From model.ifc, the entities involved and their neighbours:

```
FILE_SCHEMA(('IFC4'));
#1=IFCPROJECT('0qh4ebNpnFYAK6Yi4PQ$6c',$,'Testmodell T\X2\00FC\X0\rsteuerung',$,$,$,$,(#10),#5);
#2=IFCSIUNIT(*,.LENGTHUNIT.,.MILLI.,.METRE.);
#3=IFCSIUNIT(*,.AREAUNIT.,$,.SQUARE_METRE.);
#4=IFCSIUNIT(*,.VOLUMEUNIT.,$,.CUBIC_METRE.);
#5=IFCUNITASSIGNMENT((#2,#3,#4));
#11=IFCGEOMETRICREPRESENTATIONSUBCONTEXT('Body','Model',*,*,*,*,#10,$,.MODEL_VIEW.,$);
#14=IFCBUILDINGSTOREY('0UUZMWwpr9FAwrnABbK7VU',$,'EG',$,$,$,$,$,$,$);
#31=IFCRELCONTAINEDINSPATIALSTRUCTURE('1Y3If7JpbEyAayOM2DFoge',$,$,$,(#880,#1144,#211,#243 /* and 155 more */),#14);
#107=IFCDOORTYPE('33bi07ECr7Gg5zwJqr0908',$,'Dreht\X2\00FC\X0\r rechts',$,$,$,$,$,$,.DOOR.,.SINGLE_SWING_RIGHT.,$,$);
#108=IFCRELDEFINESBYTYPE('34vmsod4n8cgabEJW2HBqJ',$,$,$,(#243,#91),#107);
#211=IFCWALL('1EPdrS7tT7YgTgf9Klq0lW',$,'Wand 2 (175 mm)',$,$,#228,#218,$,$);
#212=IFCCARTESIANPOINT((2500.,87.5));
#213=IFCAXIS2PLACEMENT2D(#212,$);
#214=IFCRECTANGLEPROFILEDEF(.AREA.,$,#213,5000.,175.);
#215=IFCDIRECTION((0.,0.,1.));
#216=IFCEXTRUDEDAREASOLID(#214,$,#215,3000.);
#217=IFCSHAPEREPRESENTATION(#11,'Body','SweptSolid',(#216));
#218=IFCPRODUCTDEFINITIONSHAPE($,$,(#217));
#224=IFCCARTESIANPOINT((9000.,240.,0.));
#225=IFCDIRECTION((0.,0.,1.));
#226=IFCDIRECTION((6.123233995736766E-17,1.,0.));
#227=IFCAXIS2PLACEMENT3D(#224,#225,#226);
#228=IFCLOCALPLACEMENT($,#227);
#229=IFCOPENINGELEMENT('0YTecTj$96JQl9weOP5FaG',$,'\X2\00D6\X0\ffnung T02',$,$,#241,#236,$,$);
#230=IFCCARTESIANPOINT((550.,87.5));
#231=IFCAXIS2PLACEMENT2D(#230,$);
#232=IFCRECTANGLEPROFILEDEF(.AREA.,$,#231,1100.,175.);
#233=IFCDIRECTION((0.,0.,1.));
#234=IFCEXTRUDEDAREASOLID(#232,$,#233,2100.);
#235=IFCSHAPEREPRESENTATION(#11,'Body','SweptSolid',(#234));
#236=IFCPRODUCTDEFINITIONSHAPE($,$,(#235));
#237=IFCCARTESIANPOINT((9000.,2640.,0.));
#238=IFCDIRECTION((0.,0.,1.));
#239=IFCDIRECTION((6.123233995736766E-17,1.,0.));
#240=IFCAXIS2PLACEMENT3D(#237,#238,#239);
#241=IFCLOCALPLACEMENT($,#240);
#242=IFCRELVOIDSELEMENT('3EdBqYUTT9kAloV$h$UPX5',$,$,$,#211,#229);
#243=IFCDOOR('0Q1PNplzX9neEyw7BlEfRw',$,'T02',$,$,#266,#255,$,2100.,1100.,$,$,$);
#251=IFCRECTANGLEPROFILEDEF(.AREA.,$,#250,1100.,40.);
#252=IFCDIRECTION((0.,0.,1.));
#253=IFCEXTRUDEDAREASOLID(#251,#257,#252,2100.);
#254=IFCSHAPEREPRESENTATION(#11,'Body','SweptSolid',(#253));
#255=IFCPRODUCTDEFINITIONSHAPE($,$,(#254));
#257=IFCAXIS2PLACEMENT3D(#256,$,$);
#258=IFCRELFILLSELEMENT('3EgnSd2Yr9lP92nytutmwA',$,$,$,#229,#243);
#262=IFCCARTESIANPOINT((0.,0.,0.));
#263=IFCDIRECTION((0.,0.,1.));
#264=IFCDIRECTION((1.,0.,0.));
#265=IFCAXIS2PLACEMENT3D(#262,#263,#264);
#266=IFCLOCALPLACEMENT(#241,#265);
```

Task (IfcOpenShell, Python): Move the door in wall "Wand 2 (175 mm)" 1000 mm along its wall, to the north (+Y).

```python
import ifcopenshell
import ifcopenshell.api.geometry
import ifcopenshell.util.placement
import ifcopenshell.util.unit

model = ifcopenshell.open("model.ifc")
unit_scale = ifcopenshell.util.unit.calculate_unit_scale(model)

door = model.by_guid("0Q1PNplzX9neEyw7BlEfRw")
opening = door.FillsVoids[0].RelatingOpeningElement
wall = opening.VoidsElements[0].RelatingBuildingElement

wall_matrix = ifcopenshell.util.placement.get_local_placement(wall.ObjectPlacement)
shift = wall_matrix[:3, 0] * 1 / unit_scale
before = ifcopenshell.util.placement.get_local_placement(door.ObjectPlacement)[:3, 3].copy()

# The door is placed relative to its opening, so it follows when the opening moves.
matrix = ifcopenshell.util.placement.get_local_placement(opening.ObjectPlacement)
matrix[:3, 3] += shift
ifcopenshell.api.geometry.edit_object_placement(
    model, product=opening, matrix=matrix, is_si=False, should_transform_children=True
)

after = ifcopenshell.util.placement.get_local_placement(door.ObjectPlacement)[:3, 3]
print("door moved by", (after - before).round(3) + 0.0)

model.write("model_updated.ifc")
```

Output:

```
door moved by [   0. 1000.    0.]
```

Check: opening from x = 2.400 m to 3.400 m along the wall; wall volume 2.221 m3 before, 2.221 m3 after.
